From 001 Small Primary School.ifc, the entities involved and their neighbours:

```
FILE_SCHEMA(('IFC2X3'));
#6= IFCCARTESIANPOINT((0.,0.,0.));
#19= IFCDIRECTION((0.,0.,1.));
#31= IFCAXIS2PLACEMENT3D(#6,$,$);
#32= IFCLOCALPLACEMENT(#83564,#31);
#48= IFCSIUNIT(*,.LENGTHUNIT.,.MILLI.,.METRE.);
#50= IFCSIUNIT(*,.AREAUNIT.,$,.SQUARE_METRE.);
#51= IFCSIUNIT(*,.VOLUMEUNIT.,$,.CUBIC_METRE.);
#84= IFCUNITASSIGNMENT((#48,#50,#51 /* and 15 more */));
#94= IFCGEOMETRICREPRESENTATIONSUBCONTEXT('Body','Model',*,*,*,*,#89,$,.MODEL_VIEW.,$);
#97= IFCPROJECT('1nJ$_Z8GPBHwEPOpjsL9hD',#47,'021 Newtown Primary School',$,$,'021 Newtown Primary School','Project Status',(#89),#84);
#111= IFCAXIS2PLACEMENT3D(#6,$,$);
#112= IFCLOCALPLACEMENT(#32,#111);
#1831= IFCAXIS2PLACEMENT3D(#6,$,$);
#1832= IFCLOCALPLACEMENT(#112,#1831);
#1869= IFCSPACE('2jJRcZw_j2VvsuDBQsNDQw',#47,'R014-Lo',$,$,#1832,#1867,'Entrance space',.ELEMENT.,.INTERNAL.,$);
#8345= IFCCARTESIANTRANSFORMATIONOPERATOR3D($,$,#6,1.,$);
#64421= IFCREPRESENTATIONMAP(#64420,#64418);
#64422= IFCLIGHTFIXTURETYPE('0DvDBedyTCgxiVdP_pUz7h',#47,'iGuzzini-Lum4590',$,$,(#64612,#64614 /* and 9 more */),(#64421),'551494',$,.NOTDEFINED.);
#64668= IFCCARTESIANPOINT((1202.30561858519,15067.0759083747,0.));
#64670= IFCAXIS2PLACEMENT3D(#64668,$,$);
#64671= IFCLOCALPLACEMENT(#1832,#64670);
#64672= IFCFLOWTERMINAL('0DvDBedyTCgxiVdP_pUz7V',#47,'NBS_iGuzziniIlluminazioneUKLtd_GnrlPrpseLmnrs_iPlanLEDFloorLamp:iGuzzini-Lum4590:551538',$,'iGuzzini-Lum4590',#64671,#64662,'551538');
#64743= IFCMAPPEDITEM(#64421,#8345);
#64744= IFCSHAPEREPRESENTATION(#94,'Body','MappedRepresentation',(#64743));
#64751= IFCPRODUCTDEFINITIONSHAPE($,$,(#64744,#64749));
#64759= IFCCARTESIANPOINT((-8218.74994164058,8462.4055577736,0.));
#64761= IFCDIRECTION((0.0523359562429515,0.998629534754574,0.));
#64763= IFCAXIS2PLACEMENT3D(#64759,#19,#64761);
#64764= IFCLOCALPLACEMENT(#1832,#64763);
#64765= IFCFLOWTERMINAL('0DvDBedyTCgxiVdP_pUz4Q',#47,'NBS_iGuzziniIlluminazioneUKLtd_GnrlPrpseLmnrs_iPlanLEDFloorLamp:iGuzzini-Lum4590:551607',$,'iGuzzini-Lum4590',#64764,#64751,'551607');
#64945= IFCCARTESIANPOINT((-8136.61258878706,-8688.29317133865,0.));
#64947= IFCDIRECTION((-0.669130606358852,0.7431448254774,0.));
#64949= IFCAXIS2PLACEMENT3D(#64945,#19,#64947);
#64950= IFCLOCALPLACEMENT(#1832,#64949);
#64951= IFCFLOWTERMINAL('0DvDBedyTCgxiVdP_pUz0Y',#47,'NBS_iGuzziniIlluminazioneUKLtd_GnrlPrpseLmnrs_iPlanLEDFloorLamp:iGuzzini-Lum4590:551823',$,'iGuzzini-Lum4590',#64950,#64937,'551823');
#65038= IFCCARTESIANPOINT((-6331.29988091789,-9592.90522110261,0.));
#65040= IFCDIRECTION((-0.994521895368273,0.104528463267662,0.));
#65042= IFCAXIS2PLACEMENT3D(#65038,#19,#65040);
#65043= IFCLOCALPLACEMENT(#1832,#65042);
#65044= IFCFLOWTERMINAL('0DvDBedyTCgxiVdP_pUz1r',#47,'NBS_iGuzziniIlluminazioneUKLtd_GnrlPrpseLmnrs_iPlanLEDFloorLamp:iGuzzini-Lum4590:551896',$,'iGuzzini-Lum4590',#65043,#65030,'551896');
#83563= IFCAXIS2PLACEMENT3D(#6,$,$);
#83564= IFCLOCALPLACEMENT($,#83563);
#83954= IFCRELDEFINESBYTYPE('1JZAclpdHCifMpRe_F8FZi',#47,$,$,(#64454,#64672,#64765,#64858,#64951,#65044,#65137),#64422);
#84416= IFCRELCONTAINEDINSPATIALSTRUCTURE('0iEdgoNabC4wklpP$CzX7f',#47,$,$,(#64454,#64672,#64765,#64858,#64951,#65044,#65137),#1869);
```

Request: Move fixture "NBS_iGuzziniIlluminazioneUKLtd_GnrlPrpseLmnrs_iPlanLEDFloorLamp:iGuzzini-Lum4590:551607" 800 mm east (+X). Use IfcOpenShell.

```python
import ifcopenshell
import ifcopenshell.api.geometry
import ifcopenshell.util.placement
import ifcopenshell.util.unit

model = ifcopenshell.open("001 Small Primary School.ifc")
unit_scale = ifcopenshell.util.unit.calculate_unit_scale(model)

item = model.by_guid("0DvDBedyTCgxiVdP_pUz4Q")
matrix = ifcopenshell.util.placement.get_local_placement(item.ObjectPlacement)
matrix[0, 3] += 0.8 / unit_scale
ifcopenshell.api.geometry.edit_object_placement(model, product=item, matrix=matrix, is_si=False)

print(ifcopenshell.util.placement.get_local_placement(item.ObjectPlacement).round(3) + 0.0)

model.write("001 Small Primary School-out.ifc")
```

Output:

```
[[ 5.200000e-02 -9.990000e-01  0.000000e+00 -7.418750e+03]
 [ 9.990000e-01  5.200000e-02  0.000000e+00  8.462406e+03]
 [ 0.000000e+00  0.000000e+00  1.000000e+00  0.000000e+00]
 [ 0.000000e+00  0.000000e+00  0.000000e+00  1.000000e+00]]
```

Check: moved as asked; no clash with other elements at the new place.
